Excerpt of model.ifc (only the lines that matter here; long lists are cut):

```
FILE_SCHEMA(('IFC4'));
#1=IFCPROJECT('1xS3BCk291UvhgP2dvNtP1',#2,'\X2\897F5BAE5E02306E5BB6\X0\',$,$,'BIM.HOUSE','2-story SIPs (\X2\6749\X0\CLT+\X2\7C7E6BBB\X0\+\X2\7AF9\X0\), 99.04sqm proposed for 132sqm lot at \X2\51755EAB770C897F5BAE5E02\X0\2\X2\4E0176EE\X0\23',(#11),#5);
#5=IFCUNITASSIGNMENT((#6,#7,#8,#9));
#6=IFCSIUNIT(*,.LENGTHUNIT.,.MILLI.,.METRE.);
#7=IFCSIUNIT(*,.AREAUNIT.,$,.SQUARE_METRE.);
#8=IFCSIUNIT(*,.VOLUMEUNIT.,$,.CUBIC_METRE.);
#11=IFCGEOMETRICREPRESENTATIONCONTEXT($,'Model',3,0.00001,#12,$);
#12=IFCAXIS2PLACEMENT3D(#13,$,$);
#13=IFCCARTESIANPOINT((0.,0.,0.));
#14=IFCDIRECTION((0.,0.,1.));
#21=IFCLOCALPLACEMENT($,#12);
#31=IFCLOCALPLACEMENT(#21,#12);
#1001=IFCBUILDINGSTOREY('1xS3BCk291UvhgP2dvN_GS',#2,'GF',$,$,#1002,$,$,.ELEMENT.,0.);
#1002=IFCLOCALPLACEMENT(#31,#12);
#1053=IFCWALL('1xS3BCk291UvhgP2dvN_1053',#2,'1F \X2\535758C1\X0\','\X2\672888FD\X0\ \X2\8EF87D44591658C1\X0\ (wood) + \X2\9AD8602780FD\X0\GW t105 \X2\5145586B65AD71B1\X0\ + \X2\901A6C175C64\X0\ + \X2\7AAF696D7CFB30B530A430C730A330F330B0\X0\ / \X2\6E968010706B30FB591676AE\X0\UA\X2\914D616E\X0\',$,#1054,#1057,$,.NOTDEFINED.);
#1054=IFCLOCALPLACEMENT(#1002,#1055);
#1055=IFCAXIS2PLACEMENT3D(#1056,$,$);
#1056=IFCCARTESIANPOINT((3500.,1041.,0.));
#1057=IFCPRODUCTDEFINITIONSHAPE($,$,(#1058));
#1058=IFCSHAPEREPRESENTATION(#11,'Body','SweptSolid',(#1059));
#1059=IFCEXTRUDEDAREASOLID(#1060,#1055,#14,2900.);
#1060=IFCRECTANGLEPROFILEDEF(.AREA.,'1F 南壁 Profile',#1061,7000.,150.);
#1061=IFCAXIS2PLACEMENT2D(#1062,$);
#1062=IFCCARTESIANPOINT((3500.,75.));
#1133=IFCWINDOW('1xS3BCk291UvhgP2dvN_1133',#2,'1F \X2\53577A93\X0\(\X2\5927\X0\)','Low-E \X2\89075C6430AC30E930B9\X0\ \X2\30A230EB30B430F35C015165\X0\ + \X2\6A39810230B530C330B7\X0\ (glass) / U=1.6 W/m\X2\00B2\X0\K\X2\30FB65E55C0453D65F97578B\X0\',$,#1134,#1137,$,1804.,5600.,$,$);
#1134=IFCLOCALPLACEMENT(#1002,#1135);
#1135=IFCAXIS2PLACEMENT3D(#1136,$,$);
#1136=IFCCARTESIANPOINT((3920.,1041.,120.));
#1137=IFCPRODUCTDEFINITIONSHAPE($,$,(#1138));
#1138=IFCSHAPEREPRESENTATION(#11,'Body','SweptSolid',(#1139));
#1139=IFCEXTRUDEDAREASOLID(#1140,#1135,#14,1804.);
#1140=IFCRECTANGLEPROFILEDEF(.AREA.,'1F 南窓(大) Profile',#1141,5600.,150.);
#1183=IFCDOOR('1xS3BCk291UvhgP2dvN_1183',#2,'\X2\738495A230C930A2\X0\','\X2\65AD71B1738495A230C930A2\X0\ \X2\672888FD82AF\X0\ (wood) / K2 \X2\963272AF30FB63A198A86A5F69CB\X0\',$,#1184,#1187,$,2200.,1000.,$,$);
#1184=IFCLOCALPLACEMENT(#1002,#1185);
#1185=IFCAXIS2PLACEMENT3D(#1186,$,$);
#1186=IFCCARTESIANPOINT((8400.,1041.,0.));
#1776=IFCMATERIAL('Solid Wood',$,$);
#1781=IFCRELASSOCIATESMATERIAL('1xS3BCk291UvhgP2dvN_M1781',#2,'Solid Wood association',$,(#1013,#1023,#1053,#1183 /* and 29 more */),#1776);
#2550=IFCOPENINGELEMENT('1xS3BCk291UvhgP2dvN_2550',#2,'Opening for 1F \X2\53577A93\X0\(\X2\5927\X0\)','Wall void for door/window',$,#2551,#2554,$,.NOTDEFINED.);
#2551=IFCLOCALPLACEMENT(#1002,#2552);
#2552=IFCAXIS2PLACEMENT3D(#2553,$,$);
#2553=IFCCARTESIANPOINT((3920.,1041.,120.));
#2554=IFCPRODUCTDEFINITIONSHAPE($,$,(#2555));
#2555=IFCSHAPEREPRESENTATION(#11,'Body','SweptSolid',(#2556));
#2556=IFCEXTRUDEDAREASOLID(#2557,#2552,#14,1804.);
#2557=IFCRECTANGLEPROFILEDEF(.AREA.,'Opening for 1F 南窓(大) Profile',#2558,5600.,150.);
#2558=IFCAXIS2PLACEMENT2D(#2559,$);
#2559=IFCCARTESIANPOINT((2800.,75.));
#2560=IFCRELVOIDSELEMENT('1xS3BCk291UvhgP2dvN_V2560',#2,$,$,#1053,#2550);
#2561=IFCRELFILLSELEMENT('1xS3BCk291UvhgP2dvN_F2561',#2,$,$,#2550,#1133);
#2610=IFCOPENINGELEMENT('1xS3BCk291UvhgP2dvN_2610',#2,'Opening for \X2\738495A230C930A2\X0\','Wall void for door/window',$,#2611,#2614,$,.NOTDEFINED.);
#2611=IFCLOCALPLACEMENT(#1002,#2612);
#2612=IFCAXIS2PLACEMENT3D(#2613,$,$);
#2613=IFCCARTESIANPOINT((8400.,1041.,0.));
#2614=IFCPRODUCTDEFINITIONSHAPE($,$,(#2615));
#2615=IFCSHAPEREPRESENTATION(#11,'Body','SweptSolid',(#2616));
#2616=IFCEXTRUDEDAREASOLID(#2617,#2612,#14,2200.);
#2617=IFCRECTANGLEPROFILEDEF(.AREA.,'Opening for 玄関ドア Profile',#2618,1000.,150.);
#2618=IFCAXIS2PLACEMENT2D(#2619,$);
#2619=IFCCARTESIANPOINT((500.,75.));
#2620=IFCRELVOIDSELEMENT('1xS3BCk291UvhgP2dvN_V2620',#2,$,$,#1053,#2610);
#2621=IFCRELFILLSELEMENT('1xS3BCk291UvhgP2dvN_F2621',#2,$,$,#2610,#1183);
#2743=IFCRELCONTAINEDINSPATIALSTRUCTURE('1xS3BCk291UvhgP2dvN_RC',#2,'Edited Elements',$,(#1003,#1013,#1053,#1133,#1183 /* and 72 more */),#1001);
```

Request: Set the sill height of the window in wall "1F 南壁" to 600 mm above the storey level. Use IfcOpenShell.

```python
import numpy as np
import ifcopenshell
import ifcopenshell.api.geometry
import ifcopenshell.geom
import ifcopenshell.util.element
import ifcopenshell.util.placement
import ifcopenshell.util.shape
import ifcopenshell.util.unit

model = ifcopenshell.open("model.ifc")
unit_scale = ifcopenshell.util.unit.calculate_unit_scale(model)

window = model.by_guid("1xS3BCk291UvhgP2dvN_1133")
opening = window.FillsVoids[0].RelatingOpeningElement
storey = ifcopenshell.util.element.get_container(window, ifc_class="IfcBuildingStorey")
level = ifcopenshell.util.placement.get_local_placement(storey.ObjectPlacement)[2, 3]

# The opening's origin need not be at the sill, so measure its lowest point.
shape = ifcopenshell.geom.create_shape(ifcopenshell.geom.settings(), opening)
bottom = ifcopenshell.util.shape.get_shape_bottom_elevation(shape, shape.geometry) / unit_scale
dz = level + 0.6 / unit_scale - bottom

shift = np.array([0.0, 0.0, dz])
# The window is not placed relative to its opening, so move both.
for product in (opening, window):
    matrix = ifcopenshell.util.placement.get_local_placement(product.ObjectPlacement)
    matrix[:3, 3] += shift
    ifcopenshell.api.geometry.edit_object_placement(model, product=product, matrix=matrix, is_si=False)

print(f"moved by {dz * unit_scale:+.3f} m")

model.write("model_edited.ifc")
```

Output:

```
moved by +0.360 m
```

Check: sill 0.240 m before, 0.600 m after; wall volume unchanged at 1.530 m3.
